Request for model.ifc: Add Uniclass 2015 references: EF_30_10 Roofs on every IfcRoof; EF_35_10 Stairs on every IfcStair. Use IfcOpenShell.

First a look at what the model holds.

```python
import ifcopenshell

model = ifcopenshell.open("model.ifc")
print(model.schema)
print("classifications:", [c.Name for c in model.by_type("IfcClassification")])
for ifc_class in ("IfcDoor", "IfcRoof", "IfcStair", "IfcWall", "IfcWindow"):
    print(ifc_class, len(model.by_type(ifc_class)))
```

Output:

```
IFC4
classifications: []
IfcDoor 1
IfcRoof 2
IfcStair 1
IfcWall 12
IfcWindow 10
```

```python
import ifcopenshell
import ifcopenshell.api.classification

model = ifcopenshell.open("model.ifc")

system = ifcopenshell.api.classification.add_classification(model, classification="Uniclass 2015")

codes = {
    "IfcRoof": ("EF_30_10", "Roofs"),
    "IfcStair": ("EF_35_10", "Stairs"),
}
for ifc_class, (code, name) in codes.items():
    products = model.by_type(ifc_class)
    ifcopenshell.api.classification.add_reference(
        model, products=products, classification=system, identification=code, name=name
    )
    print(code, len(products))

model.write("model_updated.ifc")
```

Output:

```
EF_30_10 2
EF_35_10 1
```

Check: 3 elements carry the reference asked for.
